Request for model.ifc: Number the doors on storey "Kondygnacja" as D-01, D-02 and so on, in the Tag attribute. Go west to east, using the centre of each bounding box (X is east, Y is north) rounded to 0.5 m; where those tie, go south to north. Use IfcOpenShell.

First a look at what the model holds.

```python
import ifcopenshell
import ifcopenshell.util.element
import ifcopenshell.util.placement

model = ifcopenshell.open("model.ifc")
print(model.schema)
storey = next(s for s in model.by_type("IfcBuildingStorey") if s.Name == "Kondygnacja")
doors = [e for e in ifcopenshell.util.element.get_decomposition(storey) if e.is_a("IfcDoor")]
for e in sorted(doors, key=lambda e: e.id()):
    origin = ifcopenshell.util.placement.get_local_placement(e.ObjectPlacement)[:3, 3]
    print(e.id(), e.Tag, e.Name, origin.round(2) + 0.0, sep=" | ")
```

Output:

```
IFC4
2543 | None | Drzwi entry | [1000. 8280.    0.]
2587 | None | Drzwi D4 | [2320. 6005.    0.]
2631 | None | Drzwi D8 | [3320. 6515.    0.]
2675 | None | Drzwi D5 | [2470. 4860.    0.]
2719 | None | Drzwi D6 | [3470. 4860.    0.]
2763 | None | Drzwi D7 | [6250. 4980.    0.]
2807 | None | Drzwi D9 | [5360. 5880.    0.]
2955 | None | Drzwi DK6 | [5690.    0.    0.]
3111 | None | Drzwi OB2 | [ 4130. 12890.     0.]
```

```python
import ifcopenshell
import ifcopenshell.geom
import ifcopenshell.util.element
import ifcopenshell.util.shape

model = ifcopenshell.open("model.ifc")
settings = ifcopenshell.geom.settings()
settings.set("use-world-coords", True)


def centre(element):
    shape = ifcopenshell.geom.create_shape(settings, element)
    return ifcopenshell.util.shape.get_bbox_centroid(shape.geometry)


storey = next(s for s in model.by_type("IfcBuildingStorey") if s.Name == "Kondygnacja")
doors = [e for e in ifcopenshell.util.element.get_decomposition(storey) if e.is_a("IfcDoor")]

# Insertion points can sit at a corner or the storey origin, so sort by the geometry (in metres).
centres = {e: centre(e) for e in doors}
doors.sort(key=lambda e: (round(centres[e][0] / 0.5), centres[e][1]))

for i, e in enumerate(doors, start=1):
    number = f"D-{i:02d}"
    e.Tag = number
    print(e.id(), number)

model.write("model_edited.ifc")
```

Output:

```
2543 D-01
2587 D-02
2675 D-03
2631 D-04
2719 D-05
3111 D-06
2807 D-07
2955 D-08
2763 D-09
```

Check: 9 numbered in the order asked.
